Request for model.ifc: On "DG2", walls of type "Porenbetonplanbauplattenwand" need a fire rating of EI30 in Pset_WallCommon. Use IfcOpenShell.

First a look at what the model holds.

```python
import ifcopenshell
import ifcopenshell.util.element

model = ifcopenshell.open("model.ifc")
print(model.schema)
storey = next(s for s in model.by_type("IfcBuildingStorey") if s.Name == "DG2")
walls = [e for e in ifcopenshell.util.element.get_decomposition(storey) if e.is_a("IfcWall")]
seen = {}
for e in walls:
    element_type = ifcopenshell.util.element.get_type(e)
    key = (element_type.Name if element_type != e and element_type else None, ifcopenshell.util.element.get_pset(e, "Pset_WallCommon", "FireRating"))
    seen[key] = seen.get(key, 0) + 1
for (name, value), count in sorted(seen.items(), key=str):
    print(count, "x", name, "|", value)
```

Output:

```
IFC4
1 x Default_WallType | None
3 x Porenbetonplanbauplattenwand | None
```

```python
import ifcopenshell
import ifcopenshell.api.pset
import ifcopenshell.util.element

model = ifcopenshell.open("model.ifc")

storey = next(s for s in model.by_type("IfcBuildingStorey") if s.Name == "DG2")
walls = [e for e in ifcopenshell.util.element.get_decomposition(storey) if e.is_a("IfcWall")]

count = 0
for e in walls:
    element_type = ifcopenshell.util.element.get_type(e)
    if element_type in (None, e) or element_type.Name != "Porenbetonplanbauplattenwand":
        continue
    # add_pset returns the element's existing set when there is one.
    pset = ifcopenshell.api.pset.add_pset(model, product=e, name="Pset_WallCommon")
    ifcopenshell.api.pset.edit_pset(model, pset=pset, properties={"FireRating": "EI30"})
    count += 1

print(count, "walls updated")

model.write("model_updated.ifc")
```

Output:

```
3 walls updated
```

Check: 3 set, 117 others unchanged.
